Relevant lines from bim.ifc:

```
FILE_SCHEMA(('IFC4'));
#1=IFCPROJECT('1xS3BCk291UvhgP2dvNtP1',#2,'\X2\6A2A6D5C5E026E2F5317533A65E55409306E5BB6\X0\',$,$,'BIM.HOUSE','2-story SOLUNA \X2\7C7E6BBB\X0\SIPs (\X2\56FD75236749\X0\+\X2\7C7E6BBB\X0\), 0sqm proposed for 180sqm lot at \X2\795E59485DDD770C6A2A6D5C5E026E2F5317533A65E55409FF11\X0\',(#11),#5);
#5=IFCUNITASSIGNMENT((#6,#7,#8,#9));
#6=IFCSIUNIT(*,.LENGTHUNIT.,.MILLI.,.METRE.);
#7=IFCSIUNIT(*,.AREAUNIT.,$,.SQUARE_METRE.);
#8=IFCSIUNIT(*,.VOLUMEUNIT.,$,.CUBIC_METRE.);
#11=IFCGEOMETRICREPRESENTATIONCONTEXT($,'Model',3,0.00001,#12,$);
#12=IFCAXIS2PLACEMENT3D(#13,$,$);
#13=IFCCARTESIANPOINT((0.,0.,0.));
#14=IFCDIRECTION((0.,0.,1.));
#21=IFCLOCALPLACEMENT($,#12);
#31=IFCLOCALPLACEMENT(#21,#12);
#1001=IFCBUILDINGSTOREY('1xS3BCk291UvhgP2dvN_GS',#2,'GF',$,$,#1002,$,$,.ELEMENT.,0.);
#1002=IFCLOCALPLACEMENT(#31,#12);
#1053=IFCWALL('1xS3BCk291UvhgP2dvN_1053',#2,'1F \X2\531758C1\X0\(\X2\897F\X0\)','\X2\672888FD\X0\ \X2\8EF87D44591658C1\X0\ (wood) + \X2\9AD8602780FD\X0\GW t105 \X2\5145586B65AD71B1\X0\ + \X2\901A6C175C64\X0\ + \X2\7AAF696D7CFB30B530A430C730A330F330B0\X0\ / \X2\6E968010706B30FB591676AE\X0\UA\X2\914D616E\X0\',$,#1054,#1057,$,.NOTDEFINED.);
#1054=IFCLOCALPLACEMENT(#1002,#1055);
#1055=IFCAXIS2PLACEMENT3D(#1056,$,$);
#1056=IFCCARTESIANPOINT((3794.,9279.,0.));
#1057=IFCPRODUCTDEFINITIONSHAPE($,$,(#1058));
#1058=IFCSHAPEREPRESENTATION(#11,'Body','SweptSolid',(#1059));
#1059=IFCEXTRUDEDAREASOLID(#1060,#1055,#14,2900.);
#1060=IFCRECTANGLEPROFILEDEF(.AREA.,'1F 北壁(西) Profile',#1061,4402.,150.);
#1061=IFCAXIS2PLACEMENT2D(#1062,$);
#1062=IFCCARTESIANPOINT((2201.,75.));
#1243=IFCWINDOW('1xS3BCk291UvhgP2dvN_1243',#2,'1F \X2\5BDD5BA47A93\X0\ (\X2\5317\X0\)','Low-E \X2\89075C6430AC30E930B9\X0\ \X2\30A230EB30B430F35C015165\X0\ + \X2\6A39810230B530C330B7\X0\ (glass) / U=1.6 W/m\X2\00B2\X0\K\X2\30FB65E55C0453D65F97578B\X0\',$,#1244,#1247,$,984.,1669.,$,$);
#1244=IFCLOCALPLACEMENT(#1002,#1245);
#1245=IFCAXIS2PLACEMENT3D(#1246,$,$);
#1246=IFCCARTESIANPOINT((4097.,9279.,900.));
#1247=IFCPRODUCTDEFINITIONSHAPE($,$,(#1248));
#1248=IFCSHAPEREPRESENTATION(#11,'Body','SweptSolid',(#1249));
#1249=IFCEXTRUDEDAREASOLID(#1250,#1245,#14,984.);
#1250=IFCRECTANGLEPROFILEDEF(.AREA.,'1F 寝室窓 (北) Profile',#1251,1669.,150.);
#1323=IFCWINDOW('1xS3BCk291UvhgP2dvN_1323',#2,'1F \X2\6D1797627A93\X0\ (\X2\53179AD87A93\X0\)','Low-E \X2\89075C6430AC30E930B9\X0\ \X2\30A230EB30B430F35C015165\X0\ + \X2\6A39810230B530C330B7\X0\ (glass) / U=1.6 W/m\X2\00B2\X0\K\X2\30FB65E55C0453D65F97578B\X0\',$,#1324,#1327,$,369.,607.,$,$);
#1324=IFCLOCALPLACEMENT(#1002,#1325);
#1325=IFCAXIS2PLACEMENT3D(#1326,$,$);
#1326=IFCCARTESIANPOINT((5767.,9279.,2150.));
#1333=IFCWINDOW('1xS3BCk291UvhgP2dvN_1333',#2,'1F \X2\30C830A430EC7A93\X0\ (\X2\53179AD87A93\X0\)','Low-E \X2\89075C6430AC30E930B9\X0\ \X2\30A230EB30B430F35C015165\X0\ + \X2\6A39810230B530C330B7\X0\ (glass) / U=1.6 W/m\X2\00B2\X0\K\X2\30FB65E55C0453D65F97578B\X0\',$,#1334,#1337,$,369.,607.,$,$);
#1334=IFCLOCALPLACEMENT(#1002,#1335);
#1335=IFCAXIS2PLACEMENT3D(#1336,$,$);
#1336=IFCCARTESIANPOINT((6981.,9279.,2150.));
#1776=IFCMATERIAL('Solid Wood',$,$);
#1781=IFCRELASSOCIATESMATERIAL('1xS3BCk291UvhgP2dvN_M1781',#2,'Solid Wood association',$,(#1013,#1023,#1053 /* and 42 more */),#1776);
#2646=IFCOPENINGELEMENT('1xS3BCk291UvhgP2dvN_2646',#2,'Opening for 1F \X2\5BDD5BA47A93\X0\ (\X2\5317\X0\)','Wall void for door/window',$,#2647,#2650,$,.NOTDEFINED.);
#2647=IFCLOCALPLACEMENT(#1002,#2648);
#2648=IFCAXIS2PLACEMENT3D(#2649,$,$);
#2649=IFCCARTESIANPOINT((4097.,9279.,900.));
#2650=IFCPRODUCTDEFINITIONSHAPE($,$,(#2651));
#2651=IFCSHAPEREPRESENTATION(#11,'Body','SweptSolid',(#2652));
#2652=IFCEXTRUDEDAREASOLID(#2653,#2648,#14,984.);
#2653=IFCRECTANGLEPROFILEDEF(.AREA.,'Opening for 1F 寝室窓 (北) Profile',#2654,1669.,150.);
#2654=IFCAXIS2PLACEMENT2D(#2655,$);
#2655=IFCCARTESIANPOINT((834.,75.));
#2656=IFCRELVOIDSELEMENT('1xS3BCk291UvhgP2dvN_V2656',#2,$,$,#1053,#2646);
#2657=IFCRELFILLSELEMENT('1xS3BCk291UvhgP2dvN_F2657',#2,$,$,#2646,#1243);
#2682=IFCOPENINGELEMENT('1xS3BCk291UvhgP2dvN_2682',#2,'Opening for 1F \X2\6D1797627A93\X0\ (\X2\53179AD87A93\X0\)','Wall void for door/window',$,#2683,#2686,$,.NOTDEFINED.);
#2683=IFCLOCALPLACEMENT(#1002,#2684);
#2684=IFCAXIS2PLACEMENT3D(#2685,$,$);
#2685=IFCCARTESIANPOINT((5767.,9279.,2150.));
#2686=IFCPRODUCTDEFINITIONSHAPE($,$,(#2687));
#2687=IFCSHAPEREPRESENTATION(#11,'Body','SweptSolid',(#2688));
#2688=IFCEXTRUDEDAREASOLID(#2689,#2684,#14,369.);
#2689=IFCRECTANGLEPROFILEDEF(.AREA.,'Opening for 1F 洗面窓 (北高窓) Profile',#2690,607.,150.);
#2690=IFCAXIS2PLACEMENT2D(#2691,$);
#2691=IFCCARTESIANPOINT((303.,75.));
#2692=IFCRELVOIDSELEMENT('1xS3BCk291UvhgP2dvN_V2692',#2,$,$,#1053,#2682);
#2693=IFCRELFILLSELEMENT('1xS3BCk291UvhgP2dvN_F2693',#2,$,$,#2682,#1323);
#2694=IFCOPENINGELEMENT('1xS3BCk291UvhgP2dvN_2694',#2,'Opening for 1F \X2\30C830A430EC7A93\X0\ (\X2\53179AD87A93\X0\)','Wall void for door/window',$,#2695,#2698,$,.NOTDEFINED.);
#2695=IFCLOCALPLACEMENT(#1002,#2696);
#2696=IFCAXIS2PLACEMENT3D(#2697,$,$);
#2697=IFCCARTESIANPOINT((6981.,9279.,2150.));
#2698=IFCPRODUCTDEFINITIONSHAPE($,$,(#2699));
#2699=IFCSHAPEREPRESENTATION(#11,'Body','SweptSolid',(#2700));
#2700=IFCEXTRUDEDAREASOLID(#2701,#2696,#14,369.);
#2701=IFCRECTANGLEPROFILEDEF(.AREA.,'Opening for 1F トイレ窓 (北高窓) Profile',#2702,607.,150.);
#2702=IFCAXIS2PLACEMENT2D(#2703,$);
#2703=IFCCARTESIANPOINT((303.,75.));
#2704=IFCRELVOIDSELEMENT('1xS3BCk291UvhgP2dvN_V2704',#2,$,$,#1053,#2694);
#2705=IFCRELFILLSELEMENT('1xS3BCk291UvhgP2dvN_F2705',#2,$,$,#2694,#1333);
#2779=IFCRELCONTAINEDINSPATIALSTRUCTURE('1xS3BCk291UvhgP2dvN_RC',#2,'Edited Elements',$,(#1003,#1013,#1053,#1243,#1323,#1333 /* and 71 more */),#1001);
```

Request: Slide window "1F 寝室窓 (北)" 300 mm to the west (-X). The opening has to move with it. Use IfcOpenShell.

```python
import ifcopenshell
import ifcopenshell.api.geometry
import ifcopenshell.util.placement
import ifcopenshell.util.unit

model = ifcopenshell.open("bim.ifc")
unit_scale = ifcopenshell.util.unit.calculate_unit_scale(model)

window = model.by_id(1243)
opening = window.FillsVoids[0].RelatingOpeningElement
wall = opening.VoidsElements[0].RelatingBuildingElement

wall_matrix = ifcopenshell.util.placement.get_local_placement(wall.ObjectPlacement)
shift = wall_matrix[:3, 0] * -0.3 / unit_scale
before = ifcopenshell.util.placement.get_local_placement(window.ObjectPlacement)[:3, 3].copy()

# The window is not placed relative to its opening, so move both.
for product in (opening, window):
    matrix = ifcopenshell.util.placement.get_local_placement(product.ObjectPlacement)
    matrix[:3, 3] += shift
    ifcopenshell.api.geometry.edit_object_placement(model, product=product, matrix=matrix, is_si=False)

after = ifcopenshell.util.placement.get_local_placement(window.ObjectPlacement)[:3, 3]
print("window moved by", (after - before).round(3) + 0.0)

model.write("bim-out.ifc")
```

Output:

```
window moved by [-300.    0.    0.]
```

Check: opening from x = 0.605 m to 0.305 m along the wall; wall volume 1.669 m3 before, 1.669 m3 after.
